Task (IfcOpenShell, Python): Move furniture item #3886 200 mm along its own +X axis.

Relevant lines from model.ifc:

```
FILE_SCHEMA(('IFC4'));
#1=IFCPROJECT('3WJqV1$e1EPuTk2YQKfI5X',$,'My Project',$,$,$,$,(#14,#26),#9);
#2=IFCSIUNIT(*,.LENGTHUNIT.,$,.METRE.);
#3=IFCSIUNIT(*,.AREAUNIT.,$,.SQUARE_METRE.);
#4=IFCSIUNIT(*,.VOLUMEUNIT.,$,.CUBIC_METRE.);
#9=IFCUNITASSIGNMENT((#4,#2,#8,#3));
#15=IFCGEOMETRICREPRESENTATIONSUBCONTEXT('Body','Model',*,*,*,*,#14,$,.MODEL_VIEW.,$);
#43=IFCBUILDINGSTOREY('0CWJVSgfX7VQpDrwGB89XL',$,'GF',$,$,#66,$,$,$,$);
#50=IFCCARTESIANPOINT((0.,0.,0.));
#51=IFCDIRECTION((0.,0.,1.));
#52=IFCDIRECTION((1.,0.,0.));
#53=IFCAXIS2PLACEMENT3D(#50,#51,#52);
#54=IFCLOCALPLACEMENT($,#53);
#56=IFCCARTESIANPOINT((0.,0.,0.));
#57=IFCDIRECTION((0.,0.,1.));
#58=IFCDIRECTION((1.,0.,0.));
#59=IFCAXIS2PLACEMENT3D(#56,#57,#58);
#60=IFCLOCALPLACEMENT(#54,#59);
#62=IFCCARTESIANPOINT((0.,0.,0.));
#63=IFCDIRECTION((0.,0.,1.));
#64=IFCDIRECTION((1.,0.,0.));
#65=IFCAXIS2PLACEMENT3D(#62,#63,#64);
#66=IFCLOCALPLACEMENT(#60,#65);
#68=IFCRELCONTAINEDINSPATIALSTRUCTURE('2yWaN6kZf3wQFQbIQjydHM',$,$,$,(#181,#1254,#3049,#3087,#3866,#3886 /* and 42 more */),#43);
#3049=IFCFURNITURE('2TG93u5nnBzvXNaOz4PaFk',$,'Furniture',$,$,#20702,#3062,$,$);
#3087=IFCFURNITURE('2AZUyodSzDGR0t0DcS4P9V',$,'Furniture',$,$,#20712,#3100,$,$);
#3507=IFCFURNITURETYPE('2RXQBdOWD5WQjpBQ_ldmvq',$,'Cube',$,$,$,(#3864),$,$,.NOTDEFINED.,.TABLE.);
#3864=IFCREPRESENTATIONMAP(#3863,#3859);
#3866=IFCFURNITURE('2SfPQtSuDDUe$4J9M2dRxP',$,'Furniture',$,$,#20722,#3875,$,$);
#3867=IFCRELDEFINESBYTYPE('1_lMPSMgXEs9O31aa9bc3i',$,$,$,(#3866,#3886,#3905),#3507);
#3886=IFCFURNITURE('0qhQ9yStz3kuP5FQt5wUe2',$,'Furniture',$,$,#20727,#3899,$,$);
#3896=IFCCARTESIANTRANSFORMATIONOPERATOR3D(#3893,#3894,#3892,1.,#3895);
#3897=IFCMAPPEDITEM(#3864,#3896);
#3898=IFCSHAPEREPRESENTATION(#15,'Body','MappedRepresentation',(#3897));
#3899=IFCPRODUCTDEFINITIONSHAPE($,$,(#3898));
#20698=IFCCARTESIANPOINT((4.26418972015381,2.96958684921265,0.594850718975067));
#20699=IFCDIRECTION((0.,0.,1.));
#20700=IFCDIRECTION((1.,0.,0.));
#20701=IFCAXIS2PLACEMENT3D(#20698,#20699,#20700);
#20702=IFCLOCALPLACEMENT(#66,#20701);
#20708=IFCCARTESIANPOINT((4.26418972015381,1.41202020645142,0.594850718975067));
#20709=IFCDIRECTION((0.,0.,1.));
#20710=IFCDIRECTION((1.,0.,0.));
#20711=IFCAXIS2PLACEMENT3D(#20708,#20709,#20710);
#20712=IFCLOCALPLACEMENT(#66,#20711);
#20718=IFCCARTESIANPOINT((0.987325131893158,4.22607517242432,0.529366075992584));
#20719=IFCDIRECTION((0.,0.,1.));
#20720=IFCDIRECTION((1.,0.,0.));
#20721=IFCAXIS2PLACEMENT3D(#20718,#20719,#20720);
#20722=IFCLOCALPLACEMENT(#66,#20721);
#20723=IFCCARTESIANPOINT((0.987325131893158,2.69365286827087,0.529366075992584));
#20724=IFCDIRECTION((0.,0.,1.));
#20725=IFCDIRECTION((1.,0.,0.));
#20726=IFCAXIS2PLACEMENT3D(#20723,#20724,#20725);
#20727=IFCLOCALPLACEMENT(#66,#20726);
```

```python
import ifcopenshell
import ifcopenshell.api.geometry
import ifcopenshell.util.placement
import ifcopenshell.util.unit

model = ifcopenshell.open("model.ifc")
unit_scale = ifcopenshell.util.unit.calculate_unit_scale(model)

item = model.by_guid("0qhQ9yStz3kuP5FQt5wUe2")
matrix = ifcopenshell.util.placement.get_local_placement(item.ObjectPlacement)
matrix[:3, 3] += matrix[:3, 0] * 0.2 / unit_scale
ifcopenshell.api.geometry.edit_object_placement(model, product=item, matrix=matrix, is_si=False)

print(ifcopenshell.util.placement.get_local_placement(item.ObjectPlacement).round(3) + 0.0)

model.write("model_edited.ifc")
```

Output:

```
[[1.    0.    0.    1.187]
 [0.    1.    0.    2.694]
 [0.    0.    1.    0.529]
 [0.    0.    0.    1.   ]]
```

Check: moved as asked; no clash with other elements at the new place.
